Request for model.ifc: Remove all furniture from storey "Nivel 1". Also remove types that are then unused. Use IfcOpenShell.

First a look at what the model holds.

```python
import ifcopenshell
import ifcopenshell.util.element

model = ifcopenshell.open("model.ifc")
print(model.schema)
storey = next(s for s in model.by_type("IfcBuildingStorey") if s.Name == "Nivel 1")
furniture = [e for e in ifcopenshell.util.element.get_decomposition(storey) if e.is_a("IfcFurnishingElement")]
seen = {}
for e in furniture:
    element_type = ifcopenshell.util.element.get_type(e)
    name = element_type.Name if element_type not in (None, e) else None
    seen[name] = seen.get(name, 0) + 1
for name, count in sorted(seen.items(), key=str):
    print(count, "x", name)
```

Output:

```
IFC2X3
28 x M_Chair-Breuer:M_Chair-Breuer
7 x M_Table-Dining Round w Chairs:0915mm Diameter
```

```python
import ifcopenshell
import ifcopenshell.api.root
import ifcopenshell.util.element

model = ifcopenshell.open("model.ifc")

storey = next(s for s in model.by_type("IfcBuildingStorey") if s.Name == "Nivel 1")
furniture = [e for e in ifcopenshell.util.element.get_decomposition(storey) if e.is_a("IfcFurnishingElement")]
types = {ifcopenshell.util.element.get_type(e) for e in furniture} - {None, *furniture}

for e in furniture:
    ifcopenshell.api.root.remove_product(model, product=e)
print(len(furniture), "removed")

unused = [t for t in types if not ifcopenshell.util.element.get_types(t)]
for t in unused:
    ifcopenshell.api.root.remove_product(model, product=t)
print(len(unused), "unused types removed")

model.write("model_updated.ifc")
```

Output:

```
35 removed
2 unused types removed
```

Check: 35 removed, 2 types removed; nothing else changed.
